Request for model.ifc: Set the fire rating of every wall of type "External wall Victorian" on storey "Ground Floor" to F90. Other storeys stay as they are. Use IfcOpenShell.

First a look at what the model holds.

```python
import ifcopenshell
import ifcopenshell.util.element

model = ifcopenshell.open("model.ifc")
print(model.schema)
storey = next(s for s in model.by_type("IfcBuildingStorey") if s.Name == "Ground Floor")
walls = [e for e in ifcopenshell.util.element.get_decomposition(storey) if e.is_a("IfcWall")]
seen = {}
for e in walls:
    element_type = ifcopenshell.util.element.get_type(e)
    key = (element_type.Name if element_type != e and element_type else None, ifcopenshell.util.element.get_pset(e, "Pset_WallCommon", "FireRating"))
    seen[key] = seen.get(key, 0) + 1
for (name, value), count in sorted(seen.items(), key=str):
    print(count, "x", name, "|", value)
```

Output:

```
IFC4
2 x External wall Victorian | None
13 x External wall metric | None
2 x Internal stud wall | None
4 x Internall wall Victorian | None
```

```python
import ifcopenshell
import ifcopenshell.api.pset
import ifcopenshell.util.element

model = ifcopenshell.open("model.ifc")

storey = next(s for s in model.by_type("IfcBuildingStorey") if s.Name == "Ground Floor")
walls = [e for e in ifcopenshell.util.element.get_decomposition(storey) if e.is_a("IfcWall")]

count = 0
for e in walls:
    element_type = ifcopenshell.util.element.get_type(e)
    if element_type in (None, e) or element_type.Name != "External wall Victorian":
        continue
    # add_pset returns the element's existing set when there is one.
    pset = ifcopenshell.api.pset.add_pset(model, product=e, name="Pset_WallCommon")
    ifcopenshell.api.pset.edit_pset(model, pset=pset, properties={"FireRating": "F90"})
    count += 1

print(count, "walls updated")

model.write("model_updated.ifc")
```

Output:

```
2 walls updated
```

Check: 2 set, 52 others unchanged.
